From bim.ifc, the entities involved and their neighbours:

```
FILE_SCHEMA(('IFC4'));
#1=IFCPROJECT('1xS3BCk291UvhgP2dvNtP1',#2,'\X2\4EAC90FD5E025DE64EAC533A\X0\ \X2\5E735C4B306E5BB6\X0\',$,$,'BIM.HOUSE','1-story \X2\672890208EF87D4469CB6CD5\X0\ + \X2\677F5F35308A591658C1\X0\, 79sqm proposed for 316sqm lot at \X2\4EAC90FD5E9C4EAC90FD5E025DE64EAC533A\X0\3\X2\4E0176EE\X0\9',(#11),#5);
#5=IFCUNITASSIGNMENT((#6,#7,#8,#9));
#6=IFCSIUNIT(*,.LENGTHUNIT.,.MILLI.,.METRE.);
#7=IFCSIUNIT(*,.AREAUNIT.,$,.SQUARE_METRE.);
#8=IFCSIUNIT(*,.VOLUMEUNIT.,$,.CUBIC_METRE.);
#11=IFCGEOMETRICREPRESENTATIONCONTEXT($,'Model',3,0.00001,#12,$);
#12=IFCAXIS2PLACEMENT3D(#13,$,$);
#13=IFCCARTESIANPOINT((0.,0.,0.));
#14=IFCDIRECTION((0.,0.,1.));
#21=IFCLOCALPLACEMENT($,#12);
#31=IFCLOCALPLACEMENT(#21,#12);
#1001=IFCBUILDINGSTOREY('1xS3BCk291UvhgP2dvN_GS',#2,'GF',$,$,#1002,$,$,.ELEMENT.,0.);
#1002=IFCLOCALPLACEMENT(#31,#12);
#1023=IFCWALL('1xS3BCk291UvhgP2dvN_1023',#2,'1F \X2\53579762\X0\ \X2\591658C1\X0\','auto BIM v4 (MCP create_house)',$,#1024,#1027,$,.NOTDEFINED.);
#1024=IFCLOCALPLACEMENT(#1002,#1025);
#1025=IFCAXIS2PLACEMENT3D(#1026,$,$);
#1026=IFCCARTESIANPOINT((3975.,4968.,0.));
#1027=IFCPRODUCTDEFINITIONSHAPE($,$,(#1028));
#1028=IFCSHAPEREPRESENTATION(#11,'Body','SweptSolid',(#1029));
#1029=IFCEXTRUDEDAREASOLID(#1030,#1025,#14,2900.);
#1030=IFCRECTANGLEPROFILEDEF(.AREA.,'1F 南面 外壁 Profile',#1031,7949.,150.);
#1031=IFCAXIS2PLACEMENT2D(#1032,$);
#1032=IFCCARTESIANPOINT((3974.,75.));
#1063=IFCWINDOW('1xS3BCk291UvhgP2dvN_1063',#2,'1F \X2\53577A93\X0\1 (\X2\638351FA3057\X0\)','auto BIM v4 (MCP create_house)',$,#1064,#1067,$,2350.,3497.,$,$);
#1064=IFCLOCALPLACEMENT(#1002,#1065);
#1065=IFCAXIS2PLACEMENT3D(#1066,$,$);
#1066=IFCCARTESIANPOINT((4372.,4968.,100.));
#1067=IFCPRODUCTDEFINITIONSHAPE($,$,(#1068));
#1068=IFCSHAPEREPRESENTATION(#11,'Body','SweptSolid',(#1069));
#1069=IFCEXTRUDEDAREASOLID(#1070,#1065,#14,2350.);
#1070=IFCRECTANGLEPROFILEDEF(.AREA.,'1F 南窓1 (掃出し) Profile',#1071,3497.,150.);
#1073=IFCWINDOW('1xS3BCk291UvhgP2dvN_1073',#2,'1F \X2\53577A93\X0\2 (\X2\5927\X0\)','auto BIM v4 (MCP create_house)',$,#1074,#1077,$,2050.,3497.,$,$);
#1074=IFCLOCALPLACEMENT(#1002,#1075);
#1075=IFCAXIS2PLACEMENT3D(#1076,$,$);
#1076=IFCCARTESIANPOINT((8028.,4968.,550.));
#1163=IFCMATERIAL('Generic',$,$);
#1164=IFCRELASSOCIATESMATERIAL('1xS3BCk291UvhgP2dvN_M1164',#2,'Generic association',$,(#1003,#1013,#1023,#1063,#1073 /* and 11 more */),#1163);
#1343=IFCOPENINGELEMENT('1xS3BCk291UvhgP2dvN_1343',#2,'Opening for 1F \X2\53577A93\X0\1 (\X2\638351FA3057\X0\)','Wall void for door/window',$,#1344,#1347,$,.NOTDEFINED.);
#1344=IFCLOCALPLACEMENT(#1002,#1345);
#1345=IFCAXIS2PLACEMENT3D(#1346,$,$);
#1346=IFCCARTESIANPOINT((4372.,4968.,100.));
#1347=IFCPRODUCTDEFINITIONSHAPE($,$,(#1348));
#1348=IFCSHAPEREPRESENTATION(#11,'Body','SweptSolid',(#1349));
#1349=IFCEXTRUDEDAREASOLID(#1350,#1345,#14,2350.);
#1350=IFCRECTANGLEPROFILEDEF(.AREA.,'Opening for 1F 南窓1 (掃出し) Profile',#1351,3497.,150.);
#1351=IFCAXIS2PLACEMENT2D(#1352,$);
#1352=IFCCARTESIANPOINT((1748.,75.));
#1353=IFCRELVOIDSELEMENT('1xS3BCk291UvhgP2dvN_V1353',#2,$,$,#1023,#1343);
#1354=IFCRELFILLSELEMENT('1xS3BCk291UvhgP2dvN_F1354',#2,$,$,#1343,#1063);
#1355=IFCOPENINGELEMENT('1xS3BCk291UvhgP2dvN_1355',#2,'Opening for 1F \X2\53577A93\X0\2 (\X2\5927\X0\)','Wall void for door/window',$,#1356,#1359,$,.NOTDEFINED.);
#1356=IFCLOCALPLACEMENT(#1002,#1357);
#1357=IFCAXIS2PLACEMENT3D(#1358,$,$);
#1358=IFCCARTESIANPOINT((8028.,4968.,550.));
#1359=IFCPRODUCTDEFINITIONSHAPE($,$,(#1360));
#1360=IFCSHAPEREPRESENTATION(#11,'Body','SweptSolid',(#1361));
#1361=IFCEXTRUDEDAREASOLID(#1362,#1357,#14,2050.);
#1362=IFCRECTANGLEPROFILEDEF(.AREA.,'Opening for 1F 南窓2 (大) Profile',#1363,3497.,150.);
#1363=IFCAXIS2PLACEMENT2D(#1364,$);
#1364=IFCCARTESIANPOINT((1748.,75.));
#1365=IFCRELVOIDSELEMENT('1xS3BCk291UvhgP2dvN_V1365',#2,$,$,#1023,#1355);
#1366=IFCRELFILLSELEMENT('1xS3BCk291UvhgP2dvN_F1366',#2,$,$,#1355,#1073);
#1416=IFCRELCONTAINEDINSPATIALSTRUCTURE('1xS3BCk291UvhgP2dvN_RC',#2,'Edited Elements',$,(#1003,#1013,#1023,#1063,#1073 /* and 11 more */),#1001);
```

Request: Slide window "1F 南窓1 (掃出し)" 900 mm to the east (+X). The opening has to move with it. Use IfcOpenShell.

```python
import ifcopenshell
import ifcopenshell.api.geometry
import ifcopenshell.util.placement
import ifcopenshell.util.unit

model = ifcopenshell.open("bim.ifc")
unit_scale = ifcopenshell.util.unit.calculate_unit_scale(model)

window = model.by_id(1063)
opening = window.FillsVoids[0].RelatingOpeningElement
wall = opening.VoidsElements[0].RelatingBuildingElement

wall_matrix = ifcopenshell.util.placement.get_local_placement(wall.ObjectPlacement)
shift = wall_matrix[:3, 0] * 0.9 / unit_scale
before = ifcopenshell.util.placement.get_local_placement(window.ObjectPlacement)[:3, 3].copy()

# The window is not placed relative to its opening, so move both.
for product in (opening, window):
    matrix = ifcopenshell.util.placement.get_local_placement(product.ObjectPlacement)
    matrix[:3, 3] += shift
    ifcopenshell.api.geometry.edit_object_placement(model, product=product, matrix=matrix, is_si=False)

after = ifcopenshell.util.placement.get_local_placement(window.ObjectPlacement)[:3, 3]
print("window moved by", (after - before).round(3) + 0.0)

model.write("bim_edited.ifc")
```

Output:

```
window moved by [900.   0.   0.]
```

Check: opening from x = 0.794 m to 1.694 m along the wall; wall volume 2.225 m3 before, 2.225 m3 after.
